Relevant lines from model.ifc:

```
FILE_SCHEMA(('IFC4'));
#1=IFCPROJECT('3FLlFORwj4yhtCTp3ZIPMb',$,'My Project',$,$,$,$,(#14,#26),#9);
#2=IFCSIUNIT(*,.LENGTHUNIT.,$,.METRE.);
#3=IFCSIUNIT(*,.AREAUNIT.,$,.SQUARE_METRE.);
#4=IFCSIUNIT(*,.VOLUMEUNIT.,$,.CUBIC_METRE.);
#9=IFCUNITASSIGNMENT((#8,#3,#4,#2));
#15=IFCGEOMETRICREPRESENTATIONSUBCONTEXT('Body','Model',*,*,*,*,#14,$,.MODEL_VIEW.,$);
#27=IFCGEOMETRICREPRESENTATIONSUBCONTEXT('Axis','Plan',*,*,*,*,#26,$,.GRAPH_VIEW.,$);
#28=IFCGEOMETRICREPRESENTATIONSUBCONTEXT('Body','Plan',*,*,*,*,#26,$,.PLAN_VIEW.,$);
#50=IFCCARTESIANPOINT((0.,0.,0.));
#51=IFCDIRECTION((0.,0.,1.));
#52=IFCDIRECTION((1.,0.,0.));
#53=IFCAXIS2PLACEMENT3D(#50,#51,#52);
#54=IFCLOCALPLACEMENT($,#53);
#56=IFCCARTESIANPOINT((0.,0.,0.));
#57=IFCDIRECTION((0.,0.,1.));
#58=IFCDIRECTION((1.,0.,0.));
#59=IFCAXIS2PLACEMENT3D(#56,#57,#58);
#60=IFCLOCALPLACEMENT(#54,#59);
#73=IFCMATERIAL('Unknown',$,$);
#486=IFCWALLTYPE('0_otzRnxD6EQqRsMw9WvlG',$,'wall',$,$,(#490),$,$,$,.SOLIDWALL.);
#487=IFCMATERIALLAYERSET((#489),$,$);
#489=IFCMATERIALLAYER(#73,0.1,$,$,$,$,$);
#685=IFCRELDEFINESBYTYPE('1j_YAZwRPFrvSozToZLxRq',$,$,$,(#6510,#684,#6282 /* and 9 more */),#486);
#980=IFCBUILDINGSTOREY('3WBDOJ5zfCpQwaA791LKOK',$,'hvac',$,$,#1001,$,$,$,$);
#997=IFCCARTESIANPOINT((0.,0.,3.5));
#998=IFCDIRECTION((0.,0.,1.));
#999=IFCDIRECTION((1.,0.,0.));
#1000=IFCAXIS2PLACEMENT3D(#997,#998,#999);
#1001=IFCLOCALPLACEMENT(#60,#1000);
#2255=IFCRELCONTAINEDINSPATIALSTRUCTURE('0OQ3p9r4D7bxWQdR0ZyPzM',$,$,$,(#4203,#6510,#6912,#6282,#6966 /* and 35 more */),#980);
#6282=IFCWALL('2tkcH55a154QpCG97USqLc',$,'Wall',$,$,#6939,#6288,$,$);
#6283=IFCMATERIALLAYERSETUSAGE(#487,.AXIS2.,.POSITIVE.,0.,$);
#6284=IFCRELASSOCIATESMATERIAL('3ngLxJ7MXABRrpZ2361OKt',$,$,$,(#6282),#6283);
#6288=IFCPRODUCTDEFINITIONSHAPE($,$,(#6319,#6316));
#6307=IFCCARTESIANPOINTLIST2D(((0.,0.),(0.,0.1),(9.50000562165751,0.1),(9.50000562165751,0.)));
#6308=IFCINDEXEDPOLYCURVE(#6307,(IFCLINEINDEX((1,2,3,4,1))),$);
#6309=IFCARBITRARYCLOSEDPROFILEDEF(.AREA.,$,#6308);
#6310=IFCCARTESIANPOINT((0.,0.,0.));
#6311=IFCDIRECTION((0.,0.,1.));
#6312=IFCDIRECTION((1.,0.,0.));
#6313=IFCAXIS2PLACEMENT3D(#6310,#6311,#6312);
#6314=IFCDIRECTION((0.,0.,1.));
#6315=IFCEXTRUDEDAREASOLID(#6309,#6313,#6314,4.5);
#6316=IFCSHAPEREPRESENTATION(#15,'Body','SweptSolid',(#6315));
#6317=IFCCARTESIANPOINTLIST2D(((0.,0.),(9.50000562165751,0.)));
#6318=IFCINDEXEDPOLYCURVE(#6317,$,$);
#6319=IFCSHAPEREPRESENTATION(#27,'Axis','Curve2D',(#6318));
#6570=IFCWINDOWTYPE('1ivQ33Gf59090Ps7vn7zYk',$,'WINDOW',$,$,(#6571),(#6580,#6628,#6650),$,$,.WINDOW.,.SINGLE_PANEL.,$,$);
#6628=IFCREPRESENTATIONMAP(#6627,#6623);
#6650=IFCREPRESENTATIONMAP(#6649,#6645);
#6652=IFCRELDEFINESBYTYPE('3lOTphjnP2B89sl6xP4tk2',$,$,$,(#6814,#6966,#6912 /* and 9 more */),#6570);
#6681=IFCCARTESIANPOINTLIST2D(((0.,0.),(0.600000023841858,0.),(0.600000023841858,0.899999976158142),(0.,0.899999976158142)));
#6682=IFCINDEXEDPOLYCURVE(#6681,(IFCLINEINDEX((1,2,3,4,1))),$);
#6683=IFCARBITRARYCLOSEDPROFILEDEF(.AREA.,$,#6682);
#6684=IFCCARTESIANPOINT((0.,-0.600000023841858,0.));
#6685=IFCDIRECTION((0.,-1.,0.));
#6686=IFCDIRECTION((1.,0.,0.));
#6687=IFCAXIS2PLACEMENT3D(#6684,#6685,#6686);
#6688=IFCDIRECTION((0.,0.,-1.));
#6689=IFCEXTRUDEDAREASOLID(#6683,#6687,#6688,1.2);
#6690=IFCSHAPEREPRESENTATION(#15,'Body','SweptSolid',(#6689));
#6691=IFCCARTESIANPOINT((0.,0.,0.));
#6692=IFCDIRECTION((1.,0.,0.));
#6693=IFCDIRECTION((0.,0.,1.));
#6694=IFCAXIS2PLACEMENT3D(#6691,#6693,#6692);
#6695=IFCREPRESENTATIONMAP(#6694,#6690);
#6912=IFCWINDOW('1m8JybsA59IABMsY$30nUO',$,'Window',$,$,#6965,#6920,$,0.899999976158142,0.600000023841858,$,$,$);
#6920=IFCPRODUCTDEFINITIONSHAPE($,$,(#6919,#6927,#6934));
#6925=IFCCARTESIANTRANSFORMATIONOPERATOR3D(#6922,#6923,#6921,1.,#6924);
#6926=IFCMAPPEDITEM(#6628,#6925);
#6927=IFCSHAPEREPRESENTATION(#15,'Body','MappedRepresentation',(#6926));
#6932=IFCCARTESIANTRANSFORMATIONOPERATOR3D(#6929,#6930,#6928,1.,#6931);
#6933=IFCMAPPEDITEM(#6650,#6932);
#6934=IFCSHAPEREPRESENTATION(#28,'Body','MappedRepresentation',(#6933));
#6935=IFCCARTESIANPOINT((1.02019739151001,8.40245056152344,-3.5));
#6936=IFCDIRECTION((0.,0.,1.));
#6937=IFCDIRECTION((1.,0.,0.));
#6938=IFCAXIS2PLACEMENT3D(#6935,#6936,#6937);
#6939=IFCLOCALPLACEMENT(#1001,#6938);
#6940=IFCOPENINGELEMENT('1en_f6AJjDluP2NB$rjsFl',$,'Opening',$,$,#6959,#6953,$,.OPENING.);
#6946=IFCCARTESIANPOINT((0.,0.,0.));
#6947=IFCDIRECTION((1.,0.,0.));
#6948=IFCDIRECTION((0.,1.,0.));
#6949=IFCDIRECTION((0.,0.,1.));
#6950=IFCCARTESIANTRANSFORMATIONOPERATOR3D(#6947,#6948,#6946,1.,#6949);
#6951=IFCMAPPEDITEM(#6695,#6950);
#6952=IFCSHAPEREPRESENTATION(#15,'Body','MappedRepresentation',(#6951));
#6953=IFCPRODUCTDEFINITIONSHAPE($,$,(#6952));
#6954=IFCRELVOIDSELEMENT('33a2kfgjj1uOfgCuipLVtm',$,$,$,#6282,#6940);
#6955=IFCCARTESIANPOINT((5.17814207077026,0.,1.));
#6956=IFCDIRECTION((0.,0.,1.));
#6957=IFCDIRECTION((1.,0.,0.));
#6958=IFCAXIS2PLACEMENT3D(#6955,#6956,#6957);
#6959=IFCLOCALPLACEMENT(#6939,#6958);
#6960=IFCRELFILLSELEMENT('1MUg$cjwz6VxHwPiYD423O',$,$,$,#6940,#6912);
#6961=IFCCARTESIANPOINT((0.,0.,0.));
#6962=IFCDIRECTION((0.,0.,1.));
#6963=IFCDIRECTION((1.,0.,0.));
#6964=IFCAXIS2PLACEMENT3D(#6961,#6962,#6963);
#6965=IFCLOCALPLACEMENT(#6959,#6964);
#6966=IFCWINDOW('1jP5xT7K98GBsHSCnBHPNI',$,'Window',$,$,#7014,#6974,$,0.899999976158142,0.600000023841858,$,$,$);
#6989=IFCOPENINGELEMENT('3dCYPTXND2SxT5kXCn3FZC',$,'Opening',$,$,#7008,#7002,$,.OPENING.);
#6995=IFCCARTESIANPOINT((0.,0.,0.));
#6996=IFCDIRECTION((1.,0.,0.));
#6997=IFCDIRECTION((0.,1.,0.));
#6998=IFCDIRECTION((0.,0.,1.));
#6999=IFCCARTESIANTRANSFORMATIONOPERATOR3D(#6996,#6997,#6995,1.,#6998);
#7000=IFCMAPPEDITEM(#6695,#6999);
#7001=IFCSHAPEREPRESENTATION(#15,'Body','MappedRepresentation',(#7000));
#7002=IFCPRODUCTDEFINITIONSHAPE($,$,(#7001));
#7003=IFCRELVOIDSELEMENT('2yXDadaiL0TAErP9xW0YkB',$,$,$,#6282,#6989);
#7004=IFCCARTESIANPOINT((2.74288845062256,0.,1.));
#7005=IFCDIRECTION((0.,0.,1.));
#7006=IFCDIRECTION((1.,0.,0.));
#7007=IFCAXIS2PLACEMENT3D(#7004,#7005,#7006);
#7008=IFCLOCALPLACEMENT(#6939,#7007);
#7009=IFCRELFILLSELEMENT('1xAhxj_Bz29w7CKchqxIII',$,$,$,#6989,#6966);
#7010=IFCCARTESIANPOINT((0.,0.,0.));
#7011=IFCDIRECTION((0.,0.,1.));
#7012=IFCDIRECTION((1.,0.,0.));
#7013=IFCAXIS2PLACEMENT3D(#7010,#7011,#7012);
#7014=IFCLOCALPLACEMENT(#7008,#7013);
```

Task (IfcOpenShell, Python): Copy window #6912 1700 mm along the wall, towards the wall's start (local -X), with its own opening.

```python
import ifcopenshell
import ifcopenshell.api.feature
import ifcopenshell.api.geometry
import ifcopenshell.api.root
import ifcopenshell.geom
import ifcopenshell.util.element
import ifcopenshell.util.placement
import ifcopenshell.util.shape
import ifcopenshell.util.unit

model = ifcopenshell.open("model.ifc")
unit_scale = ifcopenshell.util.unit.calculate_unit_scale(model)
settings = ifcopenshell.geom.settings()


def volume(element):
    """Net volume in cubic metres, openings subtracted."""
    shape = ifcopenshell.geom.create_shape(settings, element)
    return ifcopenshell.util.shape.get_volume(shape.geometry)


window = model.by_guid("1m8JybsA59IABMsY$30nUO")
opening = window.FillsVoids[0].RelatingOpeningElement
wall = opening.VoidsElements[0].RelatingBuildingElement
before = volume(wall)
shift = ifcopenshell.util.placement.get_local_placement(wall.ObjectPlacement)[:3, 0] * -1.7 / unit_scale

# copy_class copies the void relationship, type, container and properties, but no geometry.
new_opening = ifcopenshell.api.root.copy_class(model, product=opening)
new_opening.Representation = ifcopenshell.util.element.copy_deep(
    model, opening.Representation, exclude=["IfcGeometricRepresentationContext", "IfcRepresentationMap"]
)
new_window = ifcopenshell.api.root.copy_class(model, product=window)
new_window.Representation = ifcopenshell.util.element.copy_deep(
    model, window.Representation, exclude=["IfcGeometricRepresentationContext", "IfcRepresentationMap"]
)
ifcopenshell.api.feature.add_filling(model, opening=new_opening, element=new_window)

for old, new in ((opening, new_opening), (window, new_window)):
    matrix = ifcopenshell.util.placement.get_local_placement(old.ObjectPlacement)
    matrix[:3, 3] += shift
    ifcopenshell.api.geometry.edit_object_placement(model, product=new, matrix=matrix, is_si=False)

after = volume(wall)

print(f"wall volume {before:.3f} -> {after:.3f} m3")

model.write("model_rev.ifc")
```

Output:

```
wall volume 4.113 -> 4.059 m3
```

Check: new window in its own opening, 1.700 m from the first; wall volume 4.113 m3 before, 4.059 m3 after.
